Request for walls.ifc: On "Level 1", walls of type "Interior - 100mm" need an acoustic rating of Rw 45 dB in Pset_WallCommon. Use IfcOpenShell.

First a look at what the model holds.

```python
import ifcopenshell
import ifcopenshell.util.element

model = ifcopenshell.open("walls.ifc")
print(model.schema)
storey = next(s for s in model.by_type("IfcBuildingStorey") if s.Name == "Level 1")
walls = [e for e in ifcopenshell.util.element.get_decomposition(storey) if e.is_a("IfcWall")]
seen = {}
for e in walls:
    element_type = ifcopenshell.util.element.get_type(e)
    key = (element_type.Name if element_type != e and element_type else None, ifcopenshell.util.element.get_pset(e, "Pset_WallCommon", "AcousticRating"))
    seen[key] = seen.get(key, 0) + 1
for (name, value), count in sorted(seen.items(), key=str):
    print(count, "x", name, "|", value)
```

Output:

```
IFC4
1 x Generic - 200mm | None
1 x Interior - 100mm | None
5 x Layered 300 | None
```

```python
import ifcopenshell
import ifcopenshell.api.pset
import ifcopenshell.util.element

model = ifcopenshell.open("walls.ifc")

storey = next(s for s in model.by_type("IfcBuildingStorey") if s.Name == "Level 1")
walls = [e for e in ifcopenshell.util.element.get_decomposition(storey) if e.is_a("IfcWall")]

count = 0
for e in walls:
    element_type = ifcopenshell.util.element.get_type(e)
    if element_type in (None, e) or element_type.Name != "Interior - 100mm":
        continue
    # add_pset returns the element's existing set when there is one.
    pset = ifcopenshell.api.pset.add_pset(model, product=e, name="Pset_WallCommon")
    ifcopenshell.api.pset.edit_pset(model, pset=pset, properties={"AcousticRating": "Rw 45 dB"})
    count += 1

print(count, "walls updated")

model.write("walls_rev.ifc")
```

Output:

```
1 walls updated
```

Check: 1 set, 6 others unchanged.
